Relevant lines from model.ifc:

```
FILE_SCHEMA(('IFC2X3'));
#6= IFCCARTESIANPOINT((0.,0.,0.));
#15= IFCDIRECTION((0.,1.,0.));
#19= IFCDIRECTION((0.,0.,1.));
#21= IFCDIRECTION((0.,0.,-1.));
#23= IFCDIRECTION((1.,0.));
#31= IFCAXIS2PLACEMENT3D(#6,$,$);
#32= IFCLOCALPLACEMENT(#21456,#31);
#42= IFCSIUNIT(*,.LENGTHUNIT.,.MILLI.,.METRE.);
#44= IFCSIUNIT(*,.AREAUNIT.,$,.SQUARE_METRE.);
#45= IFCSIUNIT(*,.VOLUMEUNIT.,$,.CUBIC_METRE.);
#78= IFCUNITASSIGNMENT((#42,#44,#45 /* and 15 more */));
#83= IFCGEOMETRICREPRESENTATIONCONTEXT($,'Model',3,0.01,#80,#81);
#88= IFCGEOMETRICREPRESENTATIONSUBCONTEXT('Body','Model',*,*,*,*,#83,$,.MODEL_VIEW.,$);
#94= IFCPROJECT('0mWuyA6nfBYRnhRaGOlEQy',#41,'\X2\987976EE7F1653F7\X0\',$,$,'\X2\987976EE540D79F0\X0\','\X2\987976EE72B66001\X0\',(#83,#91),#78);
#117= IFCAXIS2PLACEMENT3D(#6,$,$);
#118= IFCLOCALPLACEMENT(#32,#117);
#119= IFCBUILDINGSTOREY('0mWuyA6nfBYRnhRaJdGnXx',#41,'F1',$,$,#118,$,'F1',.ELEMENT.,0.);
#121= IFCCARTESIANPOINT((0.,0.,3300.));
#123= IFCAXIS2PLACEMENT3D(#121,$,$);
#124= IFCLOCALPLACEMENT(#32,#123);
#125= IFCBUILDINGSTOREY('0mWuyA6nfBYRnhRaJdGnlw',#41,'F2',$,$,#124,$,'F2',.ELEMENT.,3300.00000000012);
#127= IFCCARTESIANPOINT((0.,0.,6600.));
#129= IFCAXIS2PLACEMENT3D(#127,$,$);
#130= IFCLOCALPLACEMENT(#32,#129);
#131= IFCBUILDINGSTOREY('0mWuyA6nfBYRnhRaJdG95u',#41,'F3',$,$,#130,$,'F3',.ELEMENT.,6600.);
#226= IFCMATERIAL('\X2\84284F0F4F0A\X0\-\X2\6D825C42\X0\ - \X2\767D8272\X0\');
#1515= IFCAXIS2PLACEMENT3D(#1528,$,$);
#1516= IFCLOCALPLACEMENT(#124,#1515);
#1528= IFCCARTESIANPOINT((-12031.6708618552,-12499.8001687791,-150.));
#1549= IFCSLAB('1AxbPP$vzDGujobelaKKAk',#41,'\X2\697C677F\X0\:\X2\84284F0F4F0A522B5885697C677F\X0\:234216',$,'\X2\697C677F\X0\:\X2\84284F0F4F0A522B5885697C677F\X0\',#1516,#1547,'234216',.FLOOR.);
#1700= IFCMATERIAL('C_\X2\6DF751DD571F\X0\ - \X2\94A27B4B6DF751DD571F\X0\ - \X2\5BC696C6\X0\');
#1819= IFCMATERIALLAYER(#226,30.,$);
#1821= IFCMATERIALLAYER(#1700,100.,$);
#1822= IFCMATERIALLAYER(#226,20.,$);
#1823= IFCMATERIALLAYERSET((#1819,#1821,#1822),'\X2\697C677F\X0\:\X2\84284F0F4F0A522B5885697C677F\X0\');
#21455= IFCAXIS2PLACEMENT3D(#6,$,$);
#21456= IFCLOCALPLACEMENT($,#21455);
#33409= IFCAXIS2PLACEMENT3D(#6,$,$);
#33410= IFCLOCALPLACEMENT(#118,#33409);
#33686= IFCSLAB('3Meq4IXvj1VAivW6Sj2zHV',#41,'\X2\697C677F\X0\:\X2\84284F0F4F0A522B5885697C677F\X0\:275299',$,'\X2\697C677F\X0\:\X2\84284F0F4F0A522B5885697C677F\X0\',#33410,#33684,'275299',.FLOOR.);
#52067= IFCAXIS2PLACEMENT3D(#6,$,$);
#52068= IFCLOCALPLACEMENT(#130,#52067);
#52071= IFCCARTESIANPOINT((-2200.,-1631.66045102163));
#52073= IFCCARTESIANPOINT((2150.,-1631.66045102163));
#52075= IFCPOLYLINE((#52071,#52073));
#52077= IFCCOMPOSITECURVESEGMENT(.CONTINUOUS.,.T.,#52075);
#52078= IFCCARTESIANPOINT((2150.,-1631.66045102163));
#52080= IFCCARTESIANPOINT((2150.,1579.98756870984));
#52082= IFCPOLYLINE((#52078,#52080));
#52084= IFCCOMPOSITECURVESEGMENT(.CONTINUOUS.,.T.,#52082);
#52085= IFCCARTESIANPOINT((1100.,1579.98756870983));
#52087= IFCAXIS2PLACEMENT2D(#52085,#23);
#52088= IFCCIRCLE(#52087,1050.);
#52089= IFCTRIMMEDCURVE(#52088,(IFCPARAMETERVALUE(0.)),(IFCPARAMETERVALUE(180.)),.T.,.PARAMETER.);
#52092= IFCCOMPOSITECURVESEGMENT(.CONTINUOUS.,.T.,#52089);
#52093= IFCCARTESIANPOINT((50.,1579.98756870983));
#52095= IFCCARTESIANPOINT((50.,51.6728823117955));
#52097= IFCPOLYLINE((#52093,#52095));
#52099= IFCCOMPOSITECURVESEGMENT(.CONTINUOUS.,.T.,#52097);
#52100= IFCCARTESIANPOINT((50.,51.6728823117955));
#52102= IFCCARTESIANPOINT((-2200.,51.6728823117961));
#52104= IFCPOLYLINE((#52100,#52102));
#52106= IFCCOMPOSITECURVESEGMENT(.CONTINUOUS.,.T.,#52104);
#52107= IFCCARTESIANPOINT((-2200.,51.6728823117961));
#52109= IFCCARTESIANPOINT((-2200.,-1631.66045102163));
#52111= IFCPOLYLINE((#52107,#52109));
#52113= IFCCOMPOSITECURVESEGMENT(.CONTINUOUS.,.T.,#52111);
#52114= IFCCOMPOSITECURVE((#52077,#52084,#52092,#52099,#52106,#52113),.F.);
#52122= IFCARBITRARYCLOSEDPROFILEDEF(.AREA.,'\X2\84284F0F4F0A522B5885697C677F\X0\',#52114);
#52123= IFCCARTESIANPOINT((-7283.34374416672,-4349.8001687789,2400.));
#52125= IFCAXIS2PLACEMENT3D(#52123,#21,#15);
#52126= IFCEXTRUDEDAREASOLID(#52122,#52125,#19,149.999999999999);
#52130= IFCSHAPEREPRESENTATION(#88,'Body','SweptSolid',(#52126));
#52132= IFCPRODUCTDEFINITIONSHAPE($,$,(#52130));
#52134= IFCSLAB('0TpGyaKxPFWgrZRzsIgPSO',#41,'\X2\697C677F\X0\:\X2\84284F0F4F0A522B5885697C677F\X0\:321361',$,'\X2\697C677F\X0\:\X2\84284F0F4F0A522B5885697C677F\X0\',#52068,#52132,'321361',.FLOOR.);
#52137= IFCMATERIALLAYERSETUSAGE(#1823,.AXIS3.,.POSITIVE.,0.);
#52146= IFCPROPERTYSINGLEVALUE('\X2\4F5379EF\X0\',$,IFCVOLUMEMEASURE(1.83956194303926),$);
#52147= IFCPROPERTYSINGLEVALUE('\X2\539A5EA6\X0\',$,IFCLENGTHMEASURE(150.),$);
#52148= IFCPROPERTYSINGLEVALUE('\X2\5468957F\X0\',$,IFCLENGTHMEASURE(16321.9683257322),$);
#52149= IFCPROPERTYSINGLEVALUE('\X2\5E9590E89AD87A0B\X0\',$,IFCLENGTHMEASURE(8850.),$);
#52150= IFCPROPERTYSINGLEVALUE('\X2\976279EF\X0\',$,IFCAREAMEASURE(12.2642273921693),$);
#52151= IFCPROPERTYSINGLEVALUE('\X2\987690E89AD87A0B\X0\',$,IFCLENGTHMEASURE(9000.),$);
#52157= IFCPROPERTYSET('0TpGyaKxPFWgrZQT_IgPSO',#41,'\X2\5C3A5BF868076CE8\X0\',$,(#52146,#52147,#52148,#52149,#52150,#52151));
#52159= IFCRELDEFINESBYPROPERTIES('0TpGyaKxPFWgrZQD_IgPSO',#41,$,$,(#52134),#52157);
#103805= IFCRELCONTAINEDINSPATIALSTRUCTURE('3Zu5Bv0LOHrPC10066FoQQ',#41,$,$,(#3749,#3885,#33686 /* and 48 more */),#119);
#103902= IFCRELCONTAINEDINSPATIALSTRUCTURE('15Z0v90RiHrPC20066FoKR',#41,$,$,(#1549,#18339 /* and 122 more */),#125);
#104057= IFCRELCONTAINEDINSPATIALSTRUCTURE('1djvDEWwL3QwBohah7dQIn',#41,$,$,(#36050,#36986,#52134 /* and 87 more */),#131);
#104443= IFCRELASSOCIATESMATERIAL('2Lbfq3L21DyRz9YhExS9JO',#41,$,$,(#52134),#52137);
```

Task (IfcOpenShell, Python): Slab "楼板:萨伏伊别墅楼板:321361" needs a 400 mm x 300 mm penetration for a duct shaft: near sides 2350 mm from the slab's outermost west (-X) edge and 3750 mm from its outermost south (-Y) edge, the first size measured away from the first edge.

```python
import numpy as np
import ifcopenshell
import ifcopenshell.api.feature
import ifcopenshell.api.geometry
import ifcopenshell.api.pset
import ifcopenshell.api.root
import ifcopenshell.geom
import ifcopenshell.util.element
import ifcopenshell.util.placement
import ifcopenshell.util.representation
import ifcopenshell.util.shape
import ifcopenshell.util.unit

model = ifcopenshell.open("model.ifc")
unit_scale = ifcopenshell.util.unit.calculate_unit_scale(model)
area_scale = ifcopenshell.util.unit.calculate_unit_scale(model, "AREAUNIT")
volume_scale = ifcopenshell.util.unit.calculate_unit_scale(model, "VOLUMEUNIT")
settings = ifcopenshell.geom.settings()


def volume(element):
    """Net volume in cubic metres, openings subtracted."""
    shape = ifcopenshell.geom.create_shape(settings, element)
    return ifcopenshell.util.shape.get_volume(shape.geometry)


slab = model.by_id(52134)
before = volume(slab)

# Extent in the slab's own axes, in metres. The edges named are its -X and -Y sides.
slab_shape = ifcopenshell.geom.create_shape(settings, slab)
vertices = ifcopenshell.util.shape.get_vertices(slab_shape.geometry)
x_min, y_min, bottom = vertices.min(axis=0)
top = vertices[:, 2].max()

opening = ifcopenshell.api.root.create_entity(model, ifc_class="IfcOpeningElement", name="Duct shaft opening")
context = ifcopenshell.util.representation.get_context(model, "Model", "Body", "MODEL_VIEW")
width, depth = 0.4, 0.3
outline = [(0.0, 0.0), (width, 0.0), (width, depth), (0.0, depth), (0.0, 0.0)]
# Overshoot both faces by 50 mm so the cut is clean.
shape = ifcopenshell.api.geometry.add_slab_representation(
    model, context=context, depth=top - bottom + 0.1, polyline=outline
)
ifcopenshell.api.geometry.assign_representation(model, product=opening, representation=shape)

matrix = ifcopenshell.util.placement.get_local_placement(slab.ObjectPlacement)
matrix[:, 3] = matrix @ np.append(np.array([x_min + 2.35, y_min + 3.75, bottom - 0.05]) / unit_scale, 1.0)
ifcopenshell.api.geometry.edit_object_placement(model, product=opening, matrix=matrix, is_si=False)
ifcopenshell.api.feature.add_feature(model, feature=opening, element=slab)

after = volume(slab)

# Update the slab's stored quantities.
pset = model.by_id(ifcopenshell.util.element.get_pset(slab, "尺寸标注", should_inherit=False)["id"])
ifcopenshell.api.pset.edit_pset(model, pset=pset, properties={
    "体积": model.create_entity("IfcVolumeMeasure", after / volume_scale),
    "面积": model.create_entity("IfcAreaMeasure", after / (top - bottom) / area_scale),
})

print(f"slab volume {before:.3f} -> {after:.3f} m3")

model.write("model-out.ifc")
```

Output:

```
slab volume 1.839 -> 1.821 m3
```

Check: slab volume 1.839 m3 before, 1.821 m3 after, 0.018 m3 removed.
